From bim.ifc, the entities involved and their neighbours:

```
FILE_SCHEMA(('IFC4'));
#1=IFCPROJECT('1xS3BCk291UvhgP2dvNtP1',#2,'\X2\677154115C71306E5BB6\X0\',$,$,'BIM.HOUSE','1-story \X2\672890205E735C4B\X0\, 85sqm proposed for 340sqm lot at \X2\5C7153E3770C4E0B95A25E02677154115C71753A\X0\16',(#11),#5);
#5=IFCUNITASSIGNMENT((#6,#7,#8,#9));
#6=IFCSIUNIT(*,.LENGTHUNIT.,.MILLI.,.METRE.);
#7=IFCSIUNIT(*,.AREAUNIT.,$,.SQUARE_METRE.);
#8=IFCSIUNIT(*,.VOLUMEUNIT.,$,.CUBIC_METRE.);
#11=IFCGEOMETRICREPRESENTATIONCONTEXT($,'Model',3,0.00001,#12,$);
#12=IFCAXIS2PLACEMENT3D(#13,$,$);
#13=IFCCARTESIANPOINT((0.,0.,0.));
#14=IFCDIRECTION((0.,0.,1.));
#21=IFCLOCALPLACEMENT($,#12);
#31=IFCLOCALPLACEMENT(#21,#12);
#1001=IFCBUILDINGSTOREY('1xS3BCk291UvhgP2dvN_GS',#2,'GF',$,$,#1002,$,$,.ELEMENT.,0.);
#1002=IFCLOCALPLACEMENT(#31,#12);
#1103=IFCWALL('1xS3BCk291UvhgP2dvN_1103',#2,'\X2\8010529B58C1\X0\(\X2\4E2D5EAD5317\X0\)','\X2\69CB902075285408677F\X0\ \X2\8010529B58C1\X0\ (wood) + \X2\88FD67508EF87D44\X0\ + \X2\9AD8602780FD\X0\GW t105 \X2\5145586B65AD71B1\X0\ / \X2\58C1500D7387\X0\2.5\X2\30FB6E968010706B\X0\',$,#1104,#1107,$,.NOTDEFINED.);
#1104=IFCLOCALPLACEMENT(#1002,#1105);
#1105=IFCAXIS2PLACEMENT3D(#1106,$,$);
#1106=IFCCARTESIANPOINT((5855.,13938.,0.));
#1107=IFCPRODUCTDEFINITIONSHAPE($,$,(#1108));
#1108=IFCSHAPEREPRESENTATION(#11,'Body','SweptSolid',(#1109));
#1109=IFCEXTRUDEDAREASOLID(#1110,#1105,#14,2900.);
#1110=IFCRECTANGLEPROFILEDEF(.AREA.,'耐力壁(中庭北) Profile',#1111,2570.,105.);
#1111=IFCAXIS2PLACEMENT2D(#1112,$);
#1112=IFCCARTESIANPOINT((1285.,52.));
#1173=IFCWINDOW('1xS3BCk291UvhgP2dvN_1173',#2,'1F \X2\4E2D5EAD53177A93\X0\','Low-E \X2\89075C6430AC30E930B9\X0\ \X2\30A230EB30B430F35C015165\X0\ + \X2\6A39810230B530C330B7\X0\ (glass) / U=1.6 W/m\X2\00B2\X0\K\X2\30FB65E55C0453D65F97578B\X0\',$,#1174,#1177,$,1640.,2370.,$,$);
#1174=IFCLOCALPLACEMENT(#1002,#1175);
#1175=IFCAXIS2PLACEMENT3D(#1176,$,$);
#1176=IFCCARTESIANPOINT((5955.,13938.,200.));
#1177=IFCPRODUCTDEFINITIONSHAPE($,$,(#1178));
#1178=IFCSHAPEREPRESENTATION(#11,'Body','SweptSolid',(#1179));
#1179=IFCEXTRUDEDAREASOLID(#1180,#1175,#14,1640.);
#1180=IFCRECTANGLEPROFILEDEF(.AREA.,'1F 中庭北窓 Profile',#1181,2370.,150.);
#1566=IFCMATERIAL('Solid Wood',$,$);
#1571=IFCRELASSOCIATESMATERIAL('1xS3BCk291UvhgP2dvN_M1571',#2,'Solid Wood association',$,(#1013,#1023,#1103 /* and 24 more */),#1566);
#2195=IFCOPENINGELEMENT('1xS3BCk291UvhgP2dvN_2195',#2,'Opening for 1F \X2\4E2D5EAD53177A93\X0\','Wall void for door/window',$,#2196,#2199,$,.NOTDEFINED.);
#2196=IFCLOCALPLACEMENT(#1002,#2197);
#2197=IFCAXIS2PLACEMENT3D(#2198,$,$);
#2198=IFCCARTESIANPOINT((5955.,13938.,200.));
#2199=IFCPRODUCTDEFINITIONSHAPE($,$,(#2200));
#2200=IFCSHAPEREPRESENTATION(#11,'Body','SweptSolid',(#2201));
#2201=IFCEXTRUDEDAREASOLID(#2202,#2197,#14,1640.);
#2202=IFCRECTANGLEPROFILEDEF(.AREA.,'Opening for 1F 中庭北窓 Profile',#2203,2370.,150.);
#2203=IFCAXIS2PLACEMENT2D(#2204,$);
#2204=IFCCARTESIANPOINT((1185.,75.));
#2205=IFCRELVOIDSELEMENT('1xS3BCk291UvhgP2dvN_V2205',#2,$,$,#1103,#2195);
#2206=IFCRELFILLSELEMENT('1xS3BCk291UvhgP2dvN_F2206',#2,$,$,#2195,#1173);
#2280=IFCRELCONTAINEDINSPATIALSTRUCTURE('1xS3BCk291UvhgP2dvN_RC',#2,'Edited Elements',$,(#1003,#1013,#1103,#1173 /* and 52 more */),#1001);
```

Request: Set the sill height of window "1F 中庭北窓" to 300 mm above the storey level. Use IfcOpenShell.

```python
import numpy as np
import ifcopenshell
import ifcopenshell.api.geometry
import ifcopenshell.geom
import ifcopenshell.util.element
import ifcopenshell.util.placement
import ifcopenshell.util.shape
import ifcopenshell.util.unit

model = ifcopenshell.open("bim.ifc")
unit_scale = ifcopenshell.util.unit.calculate_unit_scale(model)

window = model.by_guid("1xS3BCk291UvhgP2dvN_1173")
opening = window.FillsVoids[0].RelatingOpeningElement
storey = ifcopenshell.util.element.get_container(window, ifc_class="IfcBuildingStorey")
level = ifcopenshell.util.placement.get_local_placement(storey.ObjectPlacement)[2, 3]

# The opening's origin need not be at the sill, so measure its lowest point.
shape = ifcopenshell.geom.create_shape(ifcopenshell.geom.settings(), opening)
bottom = ifcopenshell.util.shape.get_shape_bottom_elevation(shape, shape.geometry) / unit_scale
dz = level + 300.0 - bottom

shift = np.array([0.0, 0.0, dz])
# The window is not placed relative to its opening, so move both.
for product in (opening, window):
    matrix = ifcopenshell.util.placement.get_local_placement(product.ObjectPlacement)
    matrix[:3, 3] += shift
    ifcopenshell.api.geometry.edit_object_placement(model, product=product, matrix=matrix, is_si=False)

print(f"moved by {dz * unit_scale:+.3f} m")

model.write("bim_v2.ifc")
```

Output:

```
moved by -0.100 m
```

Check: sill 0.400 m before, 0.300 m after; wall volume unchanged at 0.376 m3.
